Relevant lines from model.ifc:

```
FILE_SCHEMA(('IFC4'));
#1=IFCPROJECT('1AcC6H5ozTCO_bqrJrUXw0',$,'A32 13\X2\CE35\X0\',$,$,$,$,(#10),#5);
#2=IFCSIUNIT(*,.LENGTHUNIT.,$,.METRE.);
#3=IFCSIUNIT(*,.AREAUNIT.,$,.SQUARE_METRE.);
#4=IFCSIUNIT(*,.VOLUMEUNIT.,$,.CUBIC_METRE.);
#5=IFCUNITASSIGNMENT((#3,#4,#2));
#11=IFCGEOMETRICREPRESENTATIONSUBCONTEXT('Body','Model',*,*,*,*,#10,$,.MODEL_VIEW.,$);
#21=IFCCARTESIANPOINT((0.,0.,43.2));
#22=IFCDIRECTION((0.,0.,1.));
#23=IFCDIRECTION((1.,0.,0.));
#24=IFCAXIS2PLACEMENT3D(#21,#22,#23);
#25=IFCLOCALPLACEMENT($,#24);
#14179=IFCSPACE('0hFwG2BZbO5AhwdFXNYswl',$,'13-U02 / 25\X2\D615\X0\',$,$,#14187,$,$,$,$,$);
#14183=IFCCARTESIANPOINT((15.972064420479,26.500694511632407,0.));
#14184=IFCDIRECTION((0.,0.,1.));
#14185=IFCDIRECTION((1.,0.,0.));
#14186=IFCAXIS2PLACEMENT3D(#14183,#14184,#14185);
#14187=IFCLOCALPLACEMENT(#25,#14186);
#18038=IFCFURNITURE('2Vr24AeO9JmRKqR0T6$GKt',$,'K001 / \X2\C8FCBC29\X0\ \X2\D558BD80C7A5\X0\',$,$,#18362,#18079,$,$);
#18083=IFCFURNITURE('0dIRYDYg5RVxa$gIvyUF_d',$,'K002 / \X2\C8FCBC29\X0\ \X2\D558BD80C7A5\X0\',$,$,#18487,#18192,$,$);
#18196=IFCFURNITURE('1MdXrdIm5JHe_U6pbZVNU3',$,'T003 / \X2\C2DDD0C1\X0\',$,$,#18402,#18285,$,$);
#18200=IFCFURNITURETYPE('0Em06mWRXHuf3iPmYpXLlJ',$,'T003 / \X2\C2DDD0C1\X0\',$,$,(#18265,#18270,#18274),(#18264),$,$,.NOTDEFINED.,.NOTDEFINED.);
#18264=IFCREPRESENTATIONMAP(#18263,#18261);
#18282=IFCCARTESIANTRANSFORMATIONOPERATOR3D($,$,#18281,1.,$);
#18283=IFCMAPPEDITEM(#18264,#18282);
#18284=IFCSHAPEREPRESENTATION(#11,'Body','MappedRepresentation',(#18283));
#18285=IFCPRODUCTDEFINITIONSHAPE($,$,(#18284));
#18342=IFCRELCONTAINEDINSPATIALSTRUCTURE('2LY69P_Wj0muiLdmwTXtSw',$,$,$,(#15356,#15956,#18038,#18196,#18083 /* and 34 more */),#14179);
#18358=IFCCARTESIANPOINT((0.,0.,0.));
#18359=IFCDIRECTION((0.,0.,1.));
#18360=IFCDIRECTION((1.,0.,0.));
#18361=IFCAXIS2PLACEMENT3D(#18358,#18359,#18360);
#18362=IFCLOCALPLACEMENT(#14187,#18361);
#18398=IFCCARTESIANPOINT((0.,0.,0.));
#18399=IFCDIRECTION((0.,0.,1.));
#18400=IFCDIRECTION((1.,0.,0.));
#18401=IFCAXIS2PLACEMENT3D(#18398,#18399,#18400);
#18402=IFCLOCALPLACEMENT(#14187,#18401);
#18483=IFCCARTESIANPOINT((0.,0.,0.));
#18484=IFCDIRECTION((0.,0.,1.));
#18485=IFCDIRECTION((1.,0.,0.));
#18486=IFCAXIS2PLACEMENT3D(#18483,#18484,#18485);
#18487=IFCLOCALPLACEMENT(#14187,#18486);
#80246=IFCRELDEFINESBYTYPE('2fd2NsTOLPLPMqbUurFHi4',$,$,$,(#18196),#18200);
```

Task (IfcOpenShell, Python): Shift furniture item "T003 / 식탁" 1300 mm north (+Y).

```python
import ifcopenshell
import ifcopenshell.api.geometry
import ifcopenshell.util.placement

model = ifcopenshell.open("model.ifc")

item = model.by_guid("1MdXrdIm5JHe_U6pbZVNU3")
matrix = ifcopenshell.util.placement.get_local_placement(item.ObjectPlacement)
matrix[1, 3] += 1.3
ifcopenshell.api.geometry.edit_object_placement(model, product=item, matrix=matrix, is_si=False)

print(ifcopenshell.util.placement.get_local_placement(item.ObjectPlacement).round(3) + 0.0)

model.write("model_rev.ifc")
```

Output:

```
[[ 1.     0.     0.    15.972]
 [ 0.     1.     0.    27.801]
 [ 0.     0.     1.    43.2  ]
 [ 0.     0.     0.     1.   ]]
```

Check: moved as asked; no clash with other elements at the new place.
